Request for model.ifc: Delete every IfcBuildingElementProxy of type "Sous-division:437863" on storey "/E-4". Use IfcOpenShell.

First a look at what the model holds.

```python
import ifcopenshell
import ifcopenshell.util.element

model = ifcopenshell.open("model.ifc")
print(model.schema)
storey = next(s for s in model.by_type("IfcBuildingStorey") if s.Name == "/E-4")
proxies = [e for e in ifcopenshell.util.element.get_decomposition(storey) if e.is_a("IfcBuildingElementProxy")]
seen = {}
for e in proxies:
    element_type = ifcopenshell.util.element.get_type(e)
    name = element_type.Name if element_type not in (None, e) else None
    seen[name] = seen.get(name, 0) + 1
for name, count in sorted(seen.items(), key=str):
    print(count, "x", name)
```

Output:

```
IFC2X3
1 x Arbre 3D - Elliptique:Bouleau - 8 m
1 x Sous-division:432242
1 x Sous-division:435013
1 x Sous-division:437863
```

```python
import ifcopenshell
import ifcopenshell.api.root
import ifcopenshell.util.element

model = ifcopenshell.open("model.ifc")

storey = next(s for s in model.by_type("IfcBuildingStorey") if s.Name == "/E-4")
proxies = [e for e in ifcopenshell.util.element.get_decomposition(storey) if e.is_a("IfcBuildingElementProxy")]
targets = [e for e in proxies if (t := ifcopenshell.util.element.get_type(e)) not in (None, e) and t.Name == "Sous-division:437863"]

for e in targets:
    ifcopenshell.api.root.remove_product(model, product=e)
print(len(targets), "removed")

model.write("model_updated.ifc")
```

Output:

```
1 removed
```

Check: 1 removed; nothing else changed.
